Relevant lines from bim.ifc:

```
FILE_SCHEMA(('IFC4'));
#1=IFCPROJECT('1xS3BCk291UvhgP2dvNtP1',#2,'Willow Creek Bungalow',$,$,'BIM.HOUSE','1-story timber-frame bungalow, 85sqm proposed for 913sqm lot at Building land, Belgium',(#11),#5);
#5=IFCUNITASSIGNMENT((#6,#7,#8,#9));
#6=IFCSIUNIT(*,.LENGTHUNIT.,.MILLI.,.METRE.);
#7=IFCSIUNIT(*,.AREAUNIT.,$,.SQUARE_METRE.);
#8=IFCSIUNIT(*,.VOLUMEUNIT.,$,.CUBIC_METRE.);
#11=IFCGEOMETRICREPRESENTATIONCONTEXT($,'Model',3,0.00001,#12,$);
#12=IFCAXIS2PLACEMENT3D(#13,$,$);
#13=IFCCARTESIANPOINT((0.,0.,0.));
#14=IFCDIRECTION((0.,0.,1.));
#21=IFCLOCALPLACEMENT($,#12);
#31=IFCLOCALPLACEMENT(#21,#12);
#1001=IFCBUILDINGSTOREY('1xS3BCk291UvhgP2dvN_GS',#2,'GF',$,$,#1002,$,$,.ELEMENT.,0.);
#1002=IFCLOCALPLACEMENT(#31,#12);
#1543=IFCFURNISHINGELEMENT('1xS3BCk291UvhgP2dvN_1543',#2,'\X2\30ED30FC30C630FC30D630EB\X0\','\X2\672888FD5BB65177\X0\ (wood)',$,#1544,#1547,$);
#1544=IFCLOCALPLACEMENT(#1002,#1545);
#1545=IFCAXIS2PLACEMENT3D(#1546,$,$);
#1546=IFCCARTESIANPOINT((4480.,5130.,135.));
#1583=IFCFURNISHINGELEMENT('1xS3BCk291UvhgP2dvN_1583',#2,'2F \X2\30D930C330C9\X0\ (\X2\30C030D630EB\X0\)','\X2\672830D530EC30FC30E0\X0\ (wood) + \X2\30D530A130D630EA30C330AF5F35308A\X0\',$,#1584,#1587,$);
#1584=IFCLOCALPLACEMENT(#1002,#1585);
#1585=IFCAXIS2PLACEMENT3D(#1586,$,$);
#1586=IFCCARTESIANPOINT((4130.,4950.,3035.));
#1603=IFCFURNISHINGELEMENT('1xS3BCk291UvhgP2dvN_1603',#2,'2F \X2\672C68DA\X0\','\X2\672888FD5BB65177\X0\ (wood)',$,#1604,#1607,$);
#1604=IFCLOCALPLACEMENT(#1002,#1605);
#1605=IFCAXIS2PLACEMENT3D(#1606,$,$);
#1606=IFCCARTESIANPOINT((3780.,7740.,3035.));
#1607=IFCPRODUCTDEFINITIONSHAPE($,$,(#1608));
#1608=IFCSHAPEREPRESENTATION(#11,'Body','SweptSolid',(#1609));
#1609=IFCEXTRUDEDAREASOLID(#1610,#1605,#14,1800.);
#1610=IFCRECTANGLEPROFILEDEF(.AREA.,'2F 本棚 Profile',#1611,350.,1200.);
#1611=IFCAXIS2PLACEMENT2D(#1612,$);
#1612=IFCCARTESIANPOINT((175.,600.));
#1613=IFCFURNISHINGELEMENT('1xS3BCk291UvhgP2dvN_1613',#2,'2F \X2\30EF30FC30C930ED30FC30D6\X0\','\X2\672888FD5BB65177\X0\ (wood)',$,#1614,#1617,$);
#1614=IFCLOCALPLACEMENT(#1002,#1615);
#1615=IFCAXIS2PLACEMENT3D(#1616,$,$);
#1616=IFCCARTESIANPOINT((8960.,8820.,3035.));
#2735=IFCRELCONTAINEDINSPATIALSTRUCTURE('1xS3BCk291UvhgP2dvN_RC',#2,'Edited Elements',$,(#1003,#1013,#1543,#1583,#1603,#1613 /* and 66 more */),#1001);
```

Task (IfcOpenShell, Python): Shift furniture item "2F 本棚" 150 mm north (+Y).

```python
import ifcopenshell
import ifcopenshell.api.geometry
import ifcopenshell.util.placement

model = ifcopenshell.open("bim.ifc")

item = model.by_guid("1xS3BCk291UvhgP2dvN_1603")
matrix = ifcopenshell.util.placement.get_local_placement(item.ObjectPlacement)
matrix[1, 3] += 150.0
ifcopenshell.api.geometry.edit_object_placement(model, product=item, matrix=matrix, is_si=False)

print(ifcopenshell.util.placement.get_local_placement(item.ObjectPlacement).round(3) + 0.0)

model.write("bim_v2.ifc")
```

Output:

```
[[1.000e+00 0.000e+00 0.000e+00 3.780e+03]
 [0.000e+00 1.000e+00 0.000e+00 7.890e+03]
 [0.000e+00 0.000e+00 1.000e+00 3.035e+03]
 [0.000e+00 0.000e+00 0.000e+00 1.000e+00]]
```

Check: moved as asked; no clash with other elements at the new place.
